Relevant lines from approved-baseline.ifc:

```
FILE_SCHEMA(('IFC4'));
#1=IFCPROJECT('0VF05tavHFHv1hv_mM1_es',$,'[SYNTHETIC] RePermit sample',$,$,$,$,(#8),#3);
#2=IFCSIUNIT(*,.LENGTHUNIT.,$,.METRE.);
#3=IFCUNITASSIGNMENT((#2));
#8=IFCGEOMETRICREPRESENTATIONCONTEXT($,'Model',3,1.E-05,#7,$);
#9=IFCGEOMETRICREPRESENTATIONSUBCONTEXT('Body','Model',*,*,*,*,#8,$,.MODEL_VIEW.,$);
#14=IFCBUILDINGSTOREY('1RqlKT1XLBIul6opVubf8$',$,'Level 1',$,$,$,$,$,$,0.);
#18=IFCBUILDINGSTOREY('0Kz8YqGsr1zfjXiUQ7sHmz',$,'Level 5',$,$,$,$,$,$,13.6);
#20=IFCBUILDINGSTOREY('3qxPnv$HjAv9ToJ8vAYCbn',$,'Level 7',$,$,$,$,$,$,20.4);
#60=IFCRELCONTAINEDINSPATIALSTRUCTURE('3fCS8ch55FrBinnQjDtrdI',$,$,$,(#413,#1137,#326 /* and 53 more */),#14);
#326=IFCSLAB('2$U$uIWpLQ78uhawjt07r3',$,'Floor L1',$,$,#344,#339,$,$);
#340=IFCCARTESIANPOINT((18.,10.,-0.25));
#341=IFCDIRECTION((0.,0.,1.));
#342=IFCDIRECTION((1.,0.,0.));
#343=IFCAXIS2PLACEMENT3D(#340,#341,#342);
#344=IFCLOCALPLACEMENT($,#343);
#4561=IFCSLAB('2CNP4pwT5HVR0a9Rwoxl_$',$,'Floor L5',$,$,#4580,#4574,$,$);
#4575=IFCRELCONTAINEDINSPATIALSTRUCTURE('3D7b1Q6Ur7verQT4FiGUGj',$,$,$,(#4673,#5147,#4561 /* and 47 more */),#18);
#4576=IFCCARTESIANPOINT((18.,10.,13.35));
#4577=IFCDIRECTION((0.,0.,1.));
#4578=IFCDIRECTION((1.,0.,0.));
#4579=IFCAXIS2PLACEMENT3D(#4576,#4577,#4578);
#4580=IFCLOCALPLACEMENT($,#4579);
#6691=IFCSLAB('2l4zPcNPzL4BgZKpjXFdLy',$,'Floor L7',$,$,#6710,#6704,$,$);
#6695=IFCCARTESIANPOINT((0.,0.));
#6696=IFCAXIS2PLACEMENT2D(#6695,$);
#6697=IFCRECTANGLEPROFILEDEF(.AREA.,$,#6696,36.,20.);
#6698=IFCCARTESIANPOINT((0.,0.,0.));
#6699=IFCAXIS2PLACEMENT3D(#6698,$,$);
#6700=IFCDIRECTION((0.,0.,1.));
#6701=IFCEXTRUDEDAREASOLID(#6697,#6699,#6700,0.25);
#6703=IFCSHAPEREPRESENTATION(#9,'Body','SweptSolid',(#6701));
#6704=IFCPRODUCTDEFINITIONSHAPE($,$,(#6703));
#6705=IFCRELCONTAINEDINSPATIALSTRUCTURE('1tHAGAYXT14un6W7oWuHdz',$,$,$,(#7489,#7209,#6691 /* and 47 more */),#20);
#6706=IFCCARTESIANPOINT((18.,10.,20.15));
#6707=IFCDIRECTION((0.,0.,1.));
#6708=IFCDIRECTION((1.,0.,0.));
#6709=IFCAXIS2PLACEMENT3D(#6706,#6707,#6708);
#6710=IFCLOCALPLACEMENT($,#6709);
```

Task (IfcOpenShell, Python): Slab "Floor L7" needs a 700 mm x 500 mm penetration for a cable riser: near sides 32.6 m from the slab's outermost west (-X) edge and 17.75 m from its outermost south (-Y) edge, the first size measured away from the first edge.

```python
import numpy as np
import ifcopenshell
import ifcopenshell.api.feature
import ifcopenshell.api.geometry
import ifcopenshell.api.root
import ifcopenshell.geom
import ifcopenshell.util.placement
import ifcopenshell.util.representation
import ifcopenshell.util.shape
import ifcopenshell.util.unit

model = ifcopenshell.open("approved-baseline.ifc")
unit_scale = ifcopenshell.util.unit.calculate_unit_scale(model)
settings = ifcopenshell.geom.settings()


def volume(element):
    """Net volume in cubic metres, openings subtracted."""
    shape = ifcopenshell.geom.create_shape(settings, element)
    return ifcopenshell.util.shape.get_volume(shape.geometry)


slab = model.by_id(6691)
before = volume(slab)

# Extent in the slab's own axes, in metres. The edges named are its -X and -Y sides.
slab_shape = ifcopenshell.geom.create_shape(settings, slab)
vertices = ifcopenshell.util.shape.get_vertices(slab_shape.geometry)
x_min, y_min, bottom = vertices.min(axis=0)
top = vertices[:, 2].max()

opening = ifcopenshell.api.root.create_entity(model, ifc_class="IfcOpeningElement", name="Cable riser opening", predefined_type="OPENING")
context = ifcopenshell.util.representation.get_context(model, "Model", "Body", "MODEL_VIEW")
width, depth = 0.7, 0.5
outline = [(0.0, 0.0), (width, 0.0), (width, depth), (0.0, depth), (0.0, 0.0)]
# Overshoot both faces by 50 mm so the cut is clean.
shape = ifcopenshell.api.geometry.add_slab_representation(
    model, context=context, depth=top - bottom + 0.1, polyline=outline
)
ifcopenshell.api.geometry.assign_representation(model, product=opening, representation=shape)

matrix = ifcopenshell.util.placement.get_local_placement(slab.ObjectPlacement)
matrix[:, 3] = matrix @ np.append(np.array([x_min + 32.6, y_min + 17.75, bottom - 0.05]) / unit_scale, 1.0)
ifcopenshell.api.geometry.edit_object_placement(model, product=opening, matrix=matrix, is_si=False)
ifcopenshell.api.feature.add_feature(model, feature=opening, element=slab)

after = volume(slab)

print(f"slab volume {before:.3f} -> {after:.3f} m3")

model.write("approved-baseline_updated.ifc")
```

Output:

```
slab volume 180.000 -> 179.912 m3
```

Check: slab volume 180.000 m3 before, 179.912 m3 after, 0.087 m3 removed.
